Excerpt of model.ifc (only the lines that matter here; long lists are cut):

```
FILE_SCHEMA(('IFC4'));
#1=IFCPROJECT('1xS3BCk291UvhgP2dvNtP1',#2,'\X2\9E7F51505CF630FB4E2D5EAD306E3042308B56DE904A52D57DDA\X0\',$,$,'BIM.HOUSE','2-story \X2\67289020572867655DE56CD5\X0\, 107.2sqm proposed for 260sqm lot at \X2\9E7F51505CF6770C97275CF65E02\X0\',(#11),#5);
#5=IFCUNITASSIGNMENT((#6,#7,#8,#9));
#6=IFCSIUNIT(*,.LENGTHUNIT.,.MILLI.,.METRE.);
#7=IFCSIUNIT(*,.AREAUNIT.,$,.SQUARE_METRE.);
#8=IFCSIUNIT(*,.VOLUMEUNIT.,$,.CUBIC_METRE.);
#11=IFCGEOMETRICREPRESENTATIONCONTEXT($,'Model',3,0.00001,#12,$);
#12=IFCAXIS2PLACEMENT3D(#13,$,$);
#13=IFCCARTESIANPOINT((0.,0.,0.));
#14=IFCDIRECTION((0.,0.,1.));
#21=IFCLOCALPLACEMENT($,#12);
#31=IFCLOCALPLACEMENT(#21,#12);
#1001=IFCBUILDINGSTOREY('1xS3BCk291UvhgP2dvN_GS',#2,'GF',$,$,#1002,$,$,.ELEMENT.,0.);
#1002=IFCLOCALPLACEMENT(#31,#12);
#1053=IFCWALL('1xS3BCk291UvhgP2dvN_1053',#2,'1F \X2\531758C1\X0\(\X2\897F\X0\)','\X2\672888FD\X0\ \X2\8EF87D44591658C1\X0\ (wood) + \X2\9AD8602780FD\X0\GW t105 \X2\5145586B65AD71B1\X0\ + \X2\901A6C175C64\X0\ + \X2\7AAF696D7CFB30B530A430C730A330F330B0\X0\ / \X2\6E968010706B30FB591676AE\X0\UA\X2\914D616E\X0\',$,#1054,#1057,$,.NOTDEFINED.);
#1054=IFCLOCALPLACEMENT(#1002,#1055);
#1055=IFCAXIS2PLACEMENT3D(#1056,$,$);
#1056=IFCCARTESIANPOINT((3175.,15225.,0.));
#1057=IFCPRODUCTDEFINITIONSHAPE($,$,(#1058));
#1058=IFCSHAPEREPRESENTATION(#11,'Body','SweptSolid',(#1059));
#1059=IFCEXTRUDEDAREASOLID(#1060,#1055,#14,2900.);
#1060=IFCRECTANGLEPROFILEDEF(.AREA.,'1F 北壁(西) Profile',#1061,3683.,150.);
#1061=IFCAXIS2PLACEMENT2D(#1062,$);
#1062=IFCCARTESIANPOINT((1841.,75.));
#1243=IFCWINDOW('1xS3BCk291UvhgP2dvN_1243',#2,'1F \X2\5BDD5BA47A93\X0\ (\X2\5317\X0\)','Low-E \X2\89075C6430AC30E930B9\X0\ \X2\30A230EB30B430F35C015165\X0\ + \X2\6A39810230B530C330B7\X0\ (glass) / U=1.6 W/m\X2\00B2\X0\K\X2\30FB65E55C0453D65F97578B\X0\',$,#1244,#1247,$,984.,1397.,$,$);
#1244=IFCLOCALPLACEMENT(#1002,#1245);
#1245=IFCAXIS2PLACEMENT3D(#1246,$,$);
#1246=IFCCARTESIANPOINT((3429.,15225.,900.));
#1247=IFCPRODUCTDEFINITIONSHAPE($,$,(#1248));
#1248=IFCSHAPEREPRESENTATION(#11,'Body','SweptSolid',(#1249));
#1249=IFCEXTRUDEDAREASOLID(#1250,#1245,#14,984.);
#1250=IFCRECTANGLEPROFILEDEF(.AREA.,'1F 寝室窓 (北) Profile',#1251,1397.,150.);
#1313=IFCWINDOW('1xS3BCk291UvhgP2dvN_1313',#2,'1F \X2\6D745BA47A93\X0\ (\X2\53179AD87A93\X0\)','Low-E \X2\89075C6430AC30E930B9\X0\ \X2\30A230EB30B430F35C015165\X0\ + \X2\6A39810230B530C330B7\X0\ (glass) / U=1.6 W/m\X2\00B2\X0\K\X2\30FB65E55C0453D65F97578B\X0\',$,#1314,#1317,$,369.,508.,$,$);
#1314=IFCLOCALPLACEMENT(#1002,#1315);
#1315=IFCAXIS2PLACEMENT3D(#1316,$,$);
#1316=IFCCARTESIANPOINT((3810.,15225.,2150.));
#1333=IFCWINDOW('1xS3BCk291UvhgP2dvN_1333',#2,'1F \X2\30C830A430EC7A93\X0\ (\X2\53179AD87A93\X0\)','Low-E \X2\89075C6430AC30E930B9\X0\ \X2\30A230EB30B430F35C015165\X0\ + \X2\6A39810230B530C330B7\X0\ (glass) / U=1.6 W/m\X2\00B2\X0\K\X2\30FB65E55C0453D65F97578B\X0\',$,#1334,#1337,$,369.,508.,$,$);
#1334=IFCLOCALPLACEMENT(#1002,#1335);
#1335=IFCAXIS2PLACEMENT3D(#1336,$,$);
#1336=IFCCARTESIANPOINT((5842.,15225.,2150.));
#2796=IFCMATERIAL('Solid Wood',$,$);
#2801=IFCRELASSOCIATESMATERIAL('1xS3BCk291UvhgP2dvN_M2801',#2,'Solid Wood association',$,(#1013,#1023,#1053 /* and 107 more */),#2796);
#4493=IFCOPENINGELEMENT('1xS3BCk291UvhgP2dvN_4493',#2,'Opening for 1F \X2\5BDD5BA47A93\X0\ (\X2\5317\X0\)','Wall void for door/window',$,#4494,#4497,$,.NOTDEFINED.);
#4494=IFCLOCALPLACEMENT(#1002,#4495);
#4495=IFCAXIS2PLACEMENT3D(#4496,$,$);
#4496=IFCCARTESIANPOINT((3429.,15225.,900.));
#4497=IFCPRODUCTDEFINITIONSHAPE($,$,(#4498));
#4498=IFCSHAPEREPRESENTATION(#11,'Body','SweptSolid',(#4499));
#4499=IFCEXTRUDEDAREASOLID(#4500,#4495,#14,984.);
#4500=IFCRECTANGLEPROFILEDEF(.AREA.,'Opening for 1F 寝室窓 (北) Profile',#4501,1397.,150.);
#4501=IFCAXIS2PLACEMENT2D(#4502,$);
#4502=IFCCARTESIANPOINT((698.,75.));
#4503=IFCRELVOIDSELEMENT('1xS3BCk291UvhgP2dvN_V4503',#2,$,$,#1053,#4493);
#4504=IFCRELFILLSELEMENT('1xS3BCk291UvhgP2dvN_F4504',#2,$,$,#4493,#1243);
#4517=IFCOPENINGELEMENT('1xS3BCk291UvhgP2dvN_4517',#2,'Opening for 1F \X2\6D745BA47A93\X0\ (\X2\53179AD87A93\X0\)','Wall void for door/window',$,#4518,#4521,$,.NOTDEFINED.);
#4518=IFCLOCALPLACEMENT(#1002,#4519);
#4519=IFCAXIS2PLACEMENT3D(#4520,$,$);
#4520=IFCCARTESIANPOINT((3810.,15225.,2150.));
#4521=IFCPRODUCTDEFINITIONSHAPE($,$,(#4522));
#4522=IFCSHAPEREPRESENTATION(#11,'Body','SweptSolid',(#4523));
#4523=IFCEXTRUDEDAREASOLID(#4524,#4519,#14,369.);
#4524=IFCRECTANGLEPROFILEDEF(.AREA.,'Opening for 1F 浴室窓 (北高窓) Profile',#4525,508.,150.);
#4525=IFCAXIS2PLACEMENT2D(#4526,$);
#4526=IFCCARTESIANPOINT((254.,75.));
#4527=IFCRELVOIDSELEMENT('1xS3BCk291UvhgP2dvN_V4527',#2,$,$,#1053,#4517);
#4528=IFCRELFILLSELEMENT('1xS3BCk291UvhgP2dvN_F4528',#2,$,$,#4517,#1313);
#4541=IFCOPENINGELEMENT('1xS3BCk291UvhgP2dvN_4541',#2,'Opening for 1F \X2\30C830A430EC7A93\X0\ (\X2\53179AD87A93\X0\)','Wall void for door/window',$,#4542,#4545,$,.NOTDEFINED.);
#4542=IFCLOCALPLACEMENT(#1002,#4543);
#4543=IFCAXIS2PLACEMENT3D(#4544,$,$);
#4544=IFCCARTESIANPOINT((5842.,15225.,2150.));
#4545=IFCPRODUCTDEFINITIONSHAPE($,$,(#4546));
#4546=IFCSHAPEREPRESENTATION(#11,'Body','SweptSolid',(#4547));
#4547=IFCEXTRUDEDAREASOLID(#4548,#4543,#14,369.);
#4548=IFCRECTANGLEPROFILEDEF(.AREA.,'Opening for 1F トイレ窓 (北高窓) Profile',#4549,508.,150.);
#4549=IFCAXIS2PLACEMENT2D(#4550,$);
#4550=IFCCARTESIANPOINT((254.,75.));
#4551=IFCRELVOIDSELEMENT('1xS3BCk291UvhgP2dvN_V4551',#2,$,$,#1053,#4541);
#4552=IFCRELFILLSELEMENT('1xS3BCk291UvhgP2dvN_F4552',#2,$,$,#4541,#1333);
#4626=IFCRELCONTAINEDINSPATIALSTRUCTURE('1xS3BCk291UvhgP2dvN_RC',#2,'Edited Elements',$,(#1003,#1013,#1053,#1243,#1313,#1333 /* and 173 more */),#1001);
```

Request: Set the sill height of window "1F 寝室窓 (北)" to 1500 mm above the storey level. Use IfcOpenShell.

```python
import numpy as np
import ifcopenshell
import ifcopenshell.api.geometry
import ifcopenshell.geom
import ifcopenshell.util.element
import ifcopenshell.util.placement
import ifcopenshell.util.shape
import ifcopenshell.util.unit

model = ifcopenshell.open("model.ifc")
unit_scale = ifcopenshell.util.unit.calculate_unit_scale(model)

window = model.by_id(1243)
opening = window.FillsVoids[0].RelatingOpeningElement
storey = ifcopenshell.util.element.get_container(window, ifc_class="IfcBuildingStorey")
level = ifcopenshell.util.placement.get_local_placement(storey.ObjectPlacement)[2, 3]

# The opening's origin need not be at the sill, so measure its lowest point.
shape = ifcopenshell.geom.create_shape(ifcopenshell.geom.settings(), opening)
bottom = ifcopenshell.util.shape.get_shape_bottom_elevation(shape, shape.geometry) / unit_scale
dz = level + 1.5 / unit_scale - bottom

shift = np.array([0.0, 0.0, dz])
# The window is not placed relative to its opening, so move both.
for product in (opening, window):
    matrix = ifcopenshell.util.placement.get_local_placement(product.ObjectPlacement)
    matrix[:3, 3] += shift
    ifcopenshell.api.geometry.edit_object_placement(model, product=product, matrix=matrix, is_si=False)

print(f"moved by {dz * unit_scale:+.3f} m")

model.write("model-out.ifc")
```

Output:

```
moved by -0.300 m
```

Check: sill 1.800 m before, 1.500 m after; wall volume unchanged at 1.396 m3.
